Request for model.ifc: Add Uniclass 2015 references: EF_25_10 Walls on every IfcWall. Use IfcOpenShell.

First a look at what the model holds.

```python
import ifcopenshell

model = ifcopenshell.open("model.ifc")
print(model.schema)
print("classifications:", [c.Name for c in model.by_type("IfcClassification")])
for ifc_class in ("IfcDoor", "IfcRoof", "IfcStair", "IfcWall", "IfcWindow"):
    print(ifc_class, len(model.by_type(ifc_class)))
```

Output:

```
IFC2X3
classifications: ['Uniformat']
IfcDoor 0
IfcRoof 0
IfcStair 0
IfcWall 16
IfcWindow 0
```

```python
import ifcopenshell
import ifcopenshell.api.classification

model = ifcopenshell.open("model.ifc")

# IFC2X3 requires Source and Edition and has no link from the project to the system.
system = model.create_entity("IfcClassification", Source="NBS", Edition="2015", Name="Uniclass 2015")

codes = {
    "IfcWall": ("EF_25_10", "Walls"),
}
for ifc_class, (code, name) in codes.items():
    products = model.by_type(ifc_class)
    ifcopenshell.api.classification.add_reference(
        model, products=products, classification=system, identification=code, name=name
    )
    print(code, len(products))

model.write("model_rev.ifc")
```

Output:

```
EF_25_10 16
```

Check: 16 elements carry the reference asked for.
